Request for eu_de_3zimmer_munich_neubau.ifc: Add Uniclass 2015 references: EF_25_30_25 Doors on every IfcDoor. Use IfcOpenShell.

First a look at what the model holds.

```python
import ifcopenshell

model = ifcopenshell.open("eu_de_3zimmer_munich_neubau.ifc")
print(model.schema)
print("classifications:", [c.Name for c in model.by_type("IfcClassification")])
for ifc_class in ("IfcDoor", "IfcRoof", "IfcStair", "IfcWall", "IfcWindow"):
    print(ifc_class, len(model.by_type(ifc_class)))
```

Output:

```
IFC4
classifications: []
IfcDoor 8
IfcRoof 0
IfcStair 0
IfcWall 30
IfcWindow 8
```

```python
import ifcopenshell
import ifcopenshell.api.classification

model = ifcopenshell.open("eu_de_3zimmer_munich_neubau.ifc")

system = ifcopenshell.api.classification.add_classification(model, classification="Uniclass 2015")

codes = {
    "IfcDoor": ("EF_25_30_25", "Doors"),
}
for ifc_class, (code, name) in codes.items():
    products = model.by_type(ifc_class)
    ifcopenshell.api.classification.add_reference(
        model, products=products, classification=system, identification=code, name=name
    )
    print(code, len(products))

model.write("eu_de_3zimmer_munich_neubau_rev.ifc")
```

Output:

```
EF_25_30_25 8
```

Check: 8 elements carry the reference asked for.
